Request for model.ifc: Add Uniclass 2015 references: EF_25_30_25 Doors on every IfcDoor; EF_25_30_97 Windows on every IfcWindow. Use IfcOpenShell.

First a look at what the model holds.

```python
import ifcopenshell

model = ifcopenshell.open("model.ifc")
print(model.schema)
print("classifications:", [c.Name for c in model.by_type("IfcClassification")])
for ifc_class in ("IfcDoor", "IfcRoof", "IfcStair", "IfcWall", "IfcWindow"):
    print(ifc_class, len(model.by_type(ifc_class)))
```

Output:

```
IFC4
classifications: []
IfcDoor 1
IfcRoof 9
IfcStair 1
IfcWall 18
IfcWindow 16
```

```python
import ifcopenshell
import ifcopenshell.api.classification

model = ifcopenshell.open("model.ifc")

system = ifcopenshell.api.classification.add_classification(model, classification="Uniclass 2015")

codes = {
    "IfcDoor": ("EF_25_30_25", "Doors"),
    "IfcWindow": ("EF_25_30_97", "Windows"),
}
for ifc_class, (code, name) in codes.items():
    products = model.by_type(ifc_class)
    ifcopenshell.api.classification.add_reference(
        model, products=products, classification=system, identification=code, name=name
    )
    print(code, len(products))

model.write("model_updated.ifc")
```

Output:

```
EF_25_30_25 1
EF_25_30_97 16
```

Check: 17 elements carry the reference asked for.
